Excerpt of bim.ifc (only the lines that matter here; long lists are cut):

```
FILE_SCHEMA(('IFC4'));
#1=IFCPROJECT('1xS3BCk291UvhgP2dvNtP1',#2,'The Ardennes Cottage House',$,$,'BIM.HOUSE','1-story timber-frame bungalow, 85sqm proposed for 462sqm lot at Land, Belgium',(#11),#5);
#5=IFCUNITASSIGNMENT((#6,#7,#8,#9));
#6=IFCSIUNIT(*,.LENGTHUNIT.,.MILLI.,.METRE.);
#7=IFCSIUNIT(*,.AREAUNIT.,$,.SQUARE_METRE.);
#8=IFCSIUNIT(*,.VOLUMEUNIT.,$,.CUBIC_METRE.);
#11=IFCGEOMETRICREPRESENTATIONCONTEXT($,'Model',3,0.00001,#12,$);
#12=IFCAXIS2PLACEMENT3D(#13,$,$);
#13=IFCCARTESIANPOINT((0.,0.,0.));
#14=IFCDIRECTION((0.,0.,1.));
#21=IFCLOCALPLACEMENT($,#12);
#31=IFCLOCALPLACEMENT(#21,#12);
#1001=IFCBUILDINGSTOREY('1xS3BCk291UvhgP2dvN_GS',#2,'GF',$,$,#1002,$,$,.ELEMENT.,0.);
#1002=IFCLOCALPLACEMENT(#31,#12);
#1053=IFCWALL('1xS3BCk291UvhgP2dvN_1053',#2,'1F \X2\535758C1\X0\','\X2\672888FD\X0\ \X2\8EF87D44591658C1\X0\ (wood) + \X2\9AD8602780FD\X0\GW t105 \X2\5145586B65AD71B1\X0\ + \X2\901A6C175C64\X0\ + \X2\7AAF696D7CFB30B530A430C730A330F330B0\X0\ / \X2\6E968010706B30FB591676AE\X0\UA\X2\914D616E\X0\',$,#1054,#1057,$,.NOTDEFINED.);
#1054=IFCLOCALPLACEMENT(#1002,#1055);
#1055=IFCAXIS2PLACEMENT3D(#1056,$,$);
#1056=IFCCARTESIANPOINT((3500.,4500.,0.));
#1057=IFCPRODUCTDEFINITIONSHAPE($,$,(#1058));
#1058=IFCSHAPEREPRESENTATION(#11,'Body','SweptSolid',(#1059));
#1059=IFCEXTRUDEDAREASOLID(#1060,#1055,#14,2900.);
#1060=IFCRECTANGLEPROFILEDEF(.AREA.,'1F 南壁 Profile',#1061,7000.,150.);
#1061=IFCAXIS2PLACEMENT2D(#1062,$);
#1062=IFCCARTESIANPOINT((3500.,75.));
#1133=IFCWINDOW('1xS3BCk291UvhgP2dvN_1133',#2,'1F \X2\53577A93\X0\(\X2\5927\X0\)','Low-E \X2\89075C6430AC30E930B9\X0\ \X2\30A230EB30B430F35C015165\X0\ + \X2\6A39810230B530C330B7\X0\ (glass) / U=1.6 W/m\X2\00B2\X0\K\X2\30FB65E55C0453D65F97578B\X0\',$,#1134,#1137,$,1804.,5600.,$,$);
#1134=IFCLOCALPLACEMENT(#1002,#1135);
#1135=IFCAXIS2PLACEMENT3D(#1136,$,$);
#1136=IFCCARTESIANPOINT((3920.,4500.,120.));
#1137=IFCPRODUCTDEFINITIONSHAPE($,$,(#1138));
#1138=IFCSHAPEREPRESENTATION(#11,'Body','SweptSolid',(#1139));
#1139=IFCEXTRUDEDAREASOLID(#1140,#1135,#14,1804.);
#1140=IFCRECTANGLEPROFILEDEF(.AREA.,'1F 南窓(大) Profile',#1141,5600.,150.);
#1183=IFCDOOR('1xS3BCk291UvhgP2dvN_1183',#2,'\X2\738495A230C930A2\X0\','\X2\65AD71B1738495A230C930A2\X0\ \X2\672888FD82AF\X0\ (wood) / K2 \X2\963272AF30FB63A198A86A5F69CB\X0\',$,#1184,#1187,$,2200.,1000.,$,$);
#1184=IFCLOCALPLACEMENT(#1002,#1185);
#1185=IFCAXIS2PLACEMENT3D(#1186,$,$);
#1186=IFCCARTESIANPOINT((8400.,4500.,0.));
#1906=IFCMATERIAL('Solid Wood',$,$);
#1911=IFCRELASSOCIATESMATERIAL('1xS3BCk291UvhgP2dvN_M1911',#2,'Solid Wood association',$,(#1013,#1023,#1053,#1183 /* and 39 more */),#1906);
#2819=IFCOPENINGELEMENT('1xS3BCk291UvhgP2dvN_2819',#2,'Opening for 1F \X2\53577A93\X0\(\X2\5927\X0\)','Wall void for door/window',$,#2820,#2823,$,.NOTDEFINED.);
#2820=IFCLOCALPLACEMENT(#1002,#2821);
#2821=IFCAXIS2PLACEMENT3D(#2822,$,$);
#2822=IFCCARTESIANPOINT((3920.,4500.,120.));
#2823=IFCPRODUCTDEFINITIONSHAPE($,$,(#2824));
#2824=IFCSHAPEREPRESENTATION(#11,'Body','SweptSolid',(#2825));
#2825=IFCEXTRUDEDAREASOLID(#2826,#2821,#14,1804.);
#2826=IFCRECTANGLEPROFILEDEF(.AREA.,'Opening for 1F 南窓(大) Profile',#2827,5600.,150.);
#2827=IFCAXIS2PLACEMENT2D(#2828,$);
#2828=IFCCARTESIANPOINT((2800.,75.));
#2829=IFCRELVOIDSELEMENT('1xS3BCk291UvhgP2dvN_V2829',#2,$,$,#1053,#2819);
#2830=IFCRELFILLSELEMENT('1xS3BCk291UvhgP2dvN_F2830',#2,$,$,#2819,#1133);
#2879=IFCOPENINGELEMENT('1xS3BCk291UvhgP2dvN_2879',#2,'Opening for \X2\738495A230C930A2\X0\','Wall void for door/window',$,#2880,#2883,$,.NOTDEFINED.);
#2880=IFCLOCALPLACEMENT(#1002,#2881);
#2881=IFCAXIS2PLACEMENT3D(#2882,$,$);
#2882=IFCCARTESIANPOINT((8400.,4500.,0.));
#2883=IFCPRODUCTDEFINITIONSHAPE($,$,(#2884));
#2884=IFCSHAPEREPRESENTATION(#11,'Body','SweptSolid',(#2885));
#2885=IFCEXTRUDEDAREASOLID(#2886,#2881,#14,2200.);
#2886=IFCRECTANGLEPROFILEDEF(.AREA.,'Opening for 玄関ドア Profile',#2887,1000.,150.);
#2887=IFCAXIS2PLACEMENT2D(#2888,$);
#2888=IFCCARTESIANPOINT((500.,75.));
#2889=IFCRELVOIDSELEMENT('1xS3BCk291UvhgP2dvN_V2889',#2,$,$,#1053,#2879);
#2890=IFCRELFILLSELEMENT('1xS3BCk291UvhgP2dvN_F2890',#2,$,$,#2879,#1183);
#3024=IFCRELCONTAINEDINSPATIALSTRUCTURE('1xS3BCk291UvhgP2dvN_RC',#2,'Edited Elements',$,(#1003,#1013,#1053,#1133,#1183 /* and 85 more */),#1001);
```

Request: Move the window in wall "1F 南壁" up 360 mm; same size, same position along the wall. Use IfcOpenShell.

```python
import numpy as np
import ifcopenshell
import ifcopenshell.api.geometry
import ifcopenshell.util.placement
import ifcopenshell.util.unit

model = ifcopenshell.open("bim.ifc")
unit_scale = ifcopenshell.util.unit.calculate_unit_scale(model)

window = model.by_guid("1xS3BCk291UvhgP2dvN_1133")
opening = window.FillsVoids[0].RelatingOpeningElement
dz = 360.0

shift = np.array([0.0, 0.0, dz])
# The window is not placed relative to its opening, so move both.
for product in (opening, window):
    matrix = ifcopenshell.util.placement.get_local_placement(product.ObjectPlacement)
    matrix[:3, 3] += shift
    ifcopenshell.api.geometry.edit_object_placement(model, product=product, matrix=matrix, is_si=False)

print(f"moved by {dz * unit_scale:+.3f} m")

model.write("bim_updated.ifc")
```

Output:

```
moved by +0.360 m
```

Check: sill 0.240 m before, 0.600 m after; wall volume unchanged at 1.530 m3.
